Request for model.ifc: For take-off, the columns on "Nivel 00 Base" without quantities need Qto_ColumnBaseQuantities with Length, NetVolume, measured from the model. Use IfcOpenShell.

First a look at what the model holds.

```python
import ifcopenshell
import ifcopenshell.util.element
import ifcopenshell.util.unit

model = ifcopenshell.open("model.ifc")
print(model.schema)
for unit_type in ("LENGTHUNIT", "AREAUNIT", "VOLUMEUNIT"):
    print(unit_type, ifcopenshell.util.unit.calculate_unit_scale(model, unit_type))
storey = next(s for s in model.by_type("IfcBuildingStorey") if s.Name == "Nivel 00 Base")
columns = [e for e in ifcopenshell.util.element.get_decomposition(storey) if e.is_a("IfcColumn")]
for e in sorted(columns, key=lambda e: e.id()):
    print(e.id(), e.is_a(), e.Name, list(ifcopenshell.util.element.get_psets(e, qtos_only=True)), sep=" | ")
```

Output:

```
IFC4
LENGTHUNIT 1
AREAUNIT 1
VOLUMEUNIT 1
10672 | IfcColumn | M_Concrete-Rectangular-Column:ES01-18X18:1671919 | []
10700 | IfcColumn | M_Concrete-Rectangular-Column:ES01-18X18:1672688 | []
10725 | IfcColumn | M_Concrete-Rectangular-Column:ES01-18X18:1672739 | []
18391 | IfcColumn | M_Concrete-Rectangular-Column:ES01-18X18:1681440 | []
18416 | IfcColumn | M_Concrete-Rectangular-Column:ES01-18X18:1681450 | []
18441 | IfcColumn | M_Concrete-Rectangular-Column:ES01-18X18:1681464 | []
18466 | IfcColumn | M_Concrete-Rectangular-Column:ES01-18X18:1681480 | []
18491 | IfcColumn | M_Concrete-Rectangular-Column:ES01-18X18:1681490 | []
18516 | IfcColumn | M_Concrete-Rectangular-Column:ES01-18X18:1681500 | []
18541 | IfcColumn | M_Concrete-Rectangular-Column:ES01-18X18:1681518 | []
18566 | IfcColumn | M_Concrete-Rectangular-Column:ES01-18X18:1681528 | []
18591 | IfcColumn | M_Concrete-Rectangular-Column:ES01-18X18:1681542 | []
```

```python
import ifcopenshell
import ifcopenshell.api.pset
import ifcopenshell.geom
import ifcopenshell.util.element
import ifcopenshell.util.shape
import ifcopenshell.util.unit

model = ifcopenshell.open("model.ifc")
unit_scale = ifcopenshell.util.unit.calculate_unit_scale(model)
volume_scale = ifcopenshell.util.unit.calculate_unit_scale(model, "VOLUMEUNIT")
settings = ifcopenshell.geom.settings()

storey = next(s for s in model.by_type("IfcBuildingStorey") if s.Name == "Nivel 00 Base")
columns = [e for e in ifcopenshell.util.element.get_decomposition(storey) if e.is_a("IfcColumn")]

for e in sorted(columns, key=lambda e: e.id()):
    if ifcopenshell.util.element.get_psets(e, qtos_only=True, should_inherit=False):
        continue
    # Geometry comes back in metres, in the element's own axes.
    shape = ifcopenshell.geom.create_shape(settings, e)
    values = {
        "Length": ifcopenshell.util.shape.get_z(shape.geometry) / unit_scale,
        "NetVolume": ifcopenshell.util.shape.get_volume(shape.geometry) / volume_scale,
    }
    qto = ifcopenshell.api.pset.add_qto(model, product=e, name="Qto_ColumnBaseQuantities")
    ifcopenshell.api.pset.edit_qto(model, qto=qto, properties=values)
    print(e.id(), {k: round(v, 3) for k, v in values.items()})

model.write("model-out.ifc")
```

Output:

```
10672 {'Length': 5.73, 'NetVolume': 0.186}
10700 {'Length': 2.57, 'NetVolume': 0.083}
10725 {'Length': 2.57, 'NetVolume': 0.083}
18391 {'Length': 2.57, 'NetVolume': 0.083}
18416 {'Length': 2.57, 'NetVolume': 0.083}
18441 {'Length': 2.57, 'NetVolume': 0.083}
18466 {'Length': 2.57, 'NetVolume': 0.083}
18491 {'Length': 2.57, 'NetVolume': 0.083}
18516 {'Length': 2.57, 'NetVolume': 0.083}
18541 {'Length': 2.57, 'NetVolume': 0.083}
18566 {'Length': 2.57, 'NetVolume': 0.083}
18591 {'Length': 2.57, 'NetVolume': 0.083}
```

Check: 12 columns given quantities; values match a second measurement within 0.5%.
